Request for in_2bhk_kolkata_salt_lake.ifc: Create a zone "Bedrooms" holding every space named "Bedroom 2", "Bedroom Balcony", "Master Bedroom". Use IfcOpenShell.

First a look at what the model holds.

```python
import ifcopenshell

model = ifcopenshell.open("in_2bhk_kolkata_salt_lake.ifc")
print(model.schema)
seen = {}
for space in model.by_type("IfcSpace"):
    seen[space.LongName] = seen.get(space.LongName, 0) + 1
for name, count in sorted(seen.items(), key=str):
    print(count, "x", name)
print("zones:", [z.Name for z in model.by_type("IfcZone")][:20])
```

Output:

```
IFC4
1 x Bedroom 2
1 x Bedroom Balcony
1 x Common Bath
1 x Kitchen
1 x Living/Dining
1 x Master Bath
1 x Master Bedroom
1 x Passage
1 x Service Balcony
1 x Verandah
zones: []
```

```python
import ifcopenshell
import ifcopenshell.api.group
import ifcopenshell.api.root

model = ifcopenshell.open("in_2bhk_kolkata_salt_lake.ifc")

names = {"Bedroom 2", "Bedroom Balcony", "Master Bedroom"}
spaces = [s for s in model.by_type("IfcSpace") if s.LongName in names]

zone = ifcopenshell.api.root.create_entity(model, ifc_class="IfcZone", name="Bedrooms")
ifcopenshell.api.group.assign_group(model, products=spaces, group=zone)
print(len(spaces), "spaces in", zone.Name)

model.write("in_2bhk_kolkata_salt_lake_rev.ifc")
```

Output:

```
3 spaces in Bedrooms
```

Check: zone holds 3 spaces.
